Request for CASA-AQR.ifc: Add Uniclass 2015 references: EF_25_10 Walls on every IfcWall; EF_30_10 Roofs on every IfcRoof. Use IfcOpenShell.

First a look at what the model holds.

```python
import ifcopenshell

model = ifcopenshell.open("CASA-AQR.ifc")
print(model.schema)
print("classifications:", [c.Name for c in model.by_type("IfcClassification")])
for ifc_class in ("IfcDoor", "IfcRoof", "IfcStair", "IfcWall", "IfcWindow"):
    print(ifc_class, len(model.by_type(ifc_class)))
```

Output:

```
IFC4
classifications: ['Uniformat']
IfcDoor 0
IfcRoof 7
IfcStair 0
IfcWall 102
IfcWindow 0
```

```python
import ifcopenshell
import ifcopenshell.api.classification

model = ifcopenshell.open("CASA-AQR.ifc")

system = ifcopenshell.api.classification.add_classification(model, classification="Uniclass 2015")

codes = {
    "IfcWall": ("EF_25_10", "Walls"),
    "IfcRoof": ("EF_30_10", "Roofs"),
}
for ifc_class, (code, name) in codes.items():
    products = model.by_type(ifc_class)
    ifcopenshell.api.classification.add_reference(
        model, products=products, classification=system, identification=code, name=name
    )
    print(code, len(products))

model.write("CASA-AQR_edited.ifc")
```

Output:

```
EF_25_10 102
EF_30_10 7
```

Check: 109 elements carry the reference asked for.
